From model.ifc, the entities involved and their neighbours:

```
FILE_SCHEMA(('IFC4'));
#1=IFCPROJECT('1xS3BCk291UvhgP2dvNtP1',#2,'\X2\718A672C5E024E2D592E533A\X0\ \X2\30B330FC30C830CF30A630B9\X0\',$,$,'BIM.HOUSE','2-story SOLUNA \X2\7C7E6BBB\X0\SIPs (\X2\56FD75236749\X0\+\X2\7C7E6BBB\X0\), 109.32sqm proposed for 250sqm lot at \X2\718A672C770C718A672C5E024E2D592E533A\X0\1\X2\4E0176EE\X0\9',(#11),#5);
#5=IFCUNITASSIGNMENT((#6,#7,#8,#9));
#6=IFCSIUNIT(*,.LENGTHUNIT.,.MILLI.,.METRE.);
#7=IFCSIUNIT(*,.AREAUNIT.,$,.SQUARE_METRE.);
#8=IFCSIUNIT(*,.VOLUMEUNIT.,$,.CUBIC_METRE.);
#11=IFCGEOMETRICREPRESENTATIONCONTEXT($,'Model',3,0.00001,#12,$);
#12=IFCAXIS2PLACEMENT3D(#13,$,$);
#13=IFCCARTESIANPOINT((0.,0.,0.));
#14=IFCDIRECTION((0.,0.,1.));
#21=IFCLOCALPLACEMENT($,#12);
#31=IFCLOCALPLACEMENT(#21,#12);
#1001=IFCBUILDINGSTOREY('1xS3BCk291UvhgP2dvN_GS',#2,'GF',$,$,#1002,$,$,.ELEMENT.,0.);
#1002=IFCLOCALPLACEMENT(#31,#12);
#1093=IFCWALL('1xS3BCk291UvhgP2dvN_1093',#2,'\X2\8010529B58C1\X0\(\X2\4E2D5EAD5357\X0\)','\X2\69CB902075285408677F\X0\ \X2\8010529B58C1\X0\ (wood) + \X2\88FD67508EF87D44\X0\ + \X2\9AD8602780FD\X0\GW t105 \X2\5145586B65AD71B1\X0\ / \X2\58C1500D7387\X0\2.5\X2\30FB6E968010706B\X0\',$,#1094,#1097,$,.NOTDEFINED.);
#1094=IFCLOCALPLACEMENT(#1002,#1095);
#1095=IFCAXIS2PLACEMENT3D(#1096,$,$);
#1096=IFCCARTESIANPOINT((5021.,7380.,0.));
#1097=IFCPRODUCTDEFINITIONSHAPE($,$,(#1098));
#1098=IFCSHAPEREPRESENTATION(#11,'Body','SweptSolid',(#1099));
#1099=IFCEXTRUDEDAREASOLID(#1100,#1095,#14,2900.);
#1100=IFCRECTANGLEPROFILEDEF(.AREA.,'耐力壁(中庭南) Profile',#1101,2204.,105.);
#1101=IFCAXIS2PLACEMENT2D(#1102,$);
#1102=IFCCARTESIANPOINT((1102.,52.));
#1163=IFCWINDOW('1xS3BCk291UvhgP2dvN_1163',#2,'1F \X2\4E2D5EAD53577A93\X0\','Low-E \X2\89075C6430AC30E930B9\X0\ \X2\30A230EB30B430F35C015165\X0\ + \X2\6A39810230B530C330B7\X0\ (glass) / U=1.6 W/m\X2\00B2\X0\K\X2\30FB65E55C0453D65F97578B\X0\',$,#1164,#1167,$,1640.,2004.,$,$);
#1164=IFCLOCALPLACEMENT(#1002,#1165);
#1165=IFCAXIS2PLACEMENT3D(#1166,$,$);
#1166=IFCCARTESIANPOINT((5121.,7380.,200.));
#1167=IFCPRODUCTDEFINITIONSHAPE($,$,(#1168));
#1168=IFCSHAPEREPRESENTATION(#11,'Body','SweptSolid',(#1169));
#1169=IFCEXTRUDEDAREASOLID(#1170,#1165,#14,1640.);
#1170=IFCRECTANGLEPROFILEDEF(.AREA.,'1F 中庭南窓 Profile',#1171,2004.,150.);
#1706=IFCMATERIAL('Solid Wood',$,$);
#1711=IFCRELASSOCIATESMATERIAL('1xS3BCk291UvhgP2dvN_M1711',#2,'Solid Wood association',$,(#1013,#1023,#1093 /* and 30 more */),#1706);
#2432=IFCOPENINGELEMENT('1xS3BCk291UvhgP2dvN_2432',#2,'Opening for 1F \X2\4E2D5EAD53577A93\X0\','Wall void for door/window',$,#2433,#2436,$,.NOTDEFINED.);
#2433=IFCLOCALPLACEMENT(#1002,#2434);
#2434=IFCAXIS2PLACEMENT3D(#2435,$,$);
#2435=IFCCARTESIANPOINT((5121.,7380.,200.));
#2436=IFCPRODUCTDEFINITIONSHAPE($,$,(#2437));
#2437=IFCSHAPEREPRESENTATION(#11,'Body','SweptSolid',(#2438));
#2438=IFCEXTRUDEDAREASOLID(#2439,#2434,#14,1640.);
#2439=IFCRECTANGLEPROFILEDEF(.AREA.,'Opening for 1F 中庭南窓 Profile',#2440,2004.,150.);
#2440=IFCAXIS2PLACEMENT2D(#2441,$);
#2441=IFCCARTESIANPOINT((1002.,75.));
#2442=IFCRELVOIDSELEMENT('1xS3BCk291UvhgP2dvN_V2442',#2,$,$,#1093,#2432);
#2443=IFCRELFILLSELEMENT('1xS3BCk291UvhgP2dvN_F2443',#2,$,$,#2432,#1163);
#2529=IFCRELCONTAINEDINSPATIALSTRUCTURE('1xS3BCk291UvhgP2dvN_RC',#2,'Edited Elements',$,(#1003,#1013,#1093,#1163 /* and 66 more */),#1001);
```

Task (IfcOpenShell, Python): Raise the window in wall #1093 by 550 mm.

```python
import numpy as np
import ifcopenshell
import ifcopenshell.api.geometry
import ifcopenshell.util.placement
import ifcopenshell.util.unit

model = ifcopenshell.open("model.ifc")
unit_scale = ifcopenshell.util.unit.calculate_unit_scale(model)

window = model.by_guid("1xS3BCk291UvhgP2dvN_1163")
opening = window.FillsVoids[0].RelatingOpeningElement
dz = 550.0

shift = np.array([0.0, 0.0, dz])
# The window is not placed relative to its opening, so move both.
for product in (opening, window):
    matrix = ifcopenshell.util.placement.get_local_placement(product.ObjectPlacement)
    matrix[:3, 3] += shift
    ifcopenshell.api.geometry.edit_object_placement(model, product=product, matrix=matrix, is_si=False)

print(f"moved by {dz * unit_scale:+.3f} m")

model.write("model_updated.ifc")
```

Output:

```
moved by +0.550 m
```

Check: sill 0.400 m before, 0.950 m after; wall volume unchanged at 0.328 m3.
